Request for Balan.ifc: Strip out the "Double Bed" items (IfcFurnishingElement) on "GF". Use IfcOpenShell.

First a look at what the model holds.

```python
import ifcopenshell
import ifcopenshell.util.element

model = ifcopenshell.open("Balan.ifc")
print(model.schema)
storey = next(s for s in model.by_type("IfcBuildingStorey") if s.Name == "GF")
furniture = [e for e in ifcopenshell.util.element.get_decomposition(storey) if e.is_a("IfcFurnishingElement")]
seen = {}
for e in furniture:
    element_type = ifcopenshell.util.element.get_type(e)
    name = element_type.Name if element_type not in (None, e) else None
    seen[name] = seen.get(name, 0) + 1
for name, count in sorted(seen.items(), key=str):
    print(count, "x", name)
```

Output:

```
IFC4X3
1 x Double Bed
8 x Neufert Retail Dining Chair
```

```python
import ifcopenshell
import ifcopenshell.api.root
import ifcopenshell.util.element

model = ifcopenshell.open("Balan.ifc")

storey = next(s for s in model.by_type("IfcBuildingStorey") if s.Name == "GF")
furniture = [e for e in ifcopenshell.util.element.get_decomposition(storey) if e.is_a("IfcFurnishingElement")]
targets = [e for e in furniture if (t := ifcopenshell.util.element.get_type(e)) not in (None, e) and t.Name == "Double Bed"]

for e in targets:
    ifcopenshell.api.root.remove_product(model, product=e)
print(len(targets), "removed")

model.write("Balan_rev.ifc")
```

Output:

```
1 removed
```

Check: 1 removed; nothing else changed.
